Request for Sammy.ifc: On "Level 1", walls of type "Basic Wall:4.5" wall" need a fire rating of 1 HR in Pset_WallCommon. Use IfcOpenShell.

First a look at what the model holds.

```python
import ifcopenshell
import ifcopenshell.util.element

model = ifcopenshell.open("Sammy.ifc")
print(model.schema)
storey = next(s for s in model.by_type("IfcBuildingStorey") if s.Name == "Level 1")
walls = [e for e in ifcopenshell.util.element.get_decomposition(storey) if e.is_a("IfcWall")]
seen = {}
for e in walls:
    element_type = ifcopenshell.util.element.get_type(e)
    key = (element_type.Name if element_type != e and element_type else None, ifcopenshell.util.element.get_pset(e, "Pset_WallCommon", "FireRating"))
    seen[key] = seen.get(key, 0) + 1
for (name, value), count in sorted(seen.items(), key=str):
    print(count, "x", name, "|", value)
```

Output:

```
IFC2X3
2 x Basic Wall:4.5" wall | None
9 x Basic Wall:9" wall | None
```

```python
import ifcopenshell
import ifcopenshell.api.pset
import ifcopenshell.util.element

model = ifcopenshell.open("Sammy.ifc")

storey = next(s for s in model.by_type("IfcBuildingStorey") if s.Name == "Level 1")
walls = [e for e in ifcopenshell.util.element.get_decomposition(storey) if e.is_a("IfcWall")]

count = 0
for e in walls:
    element_type = ifcopenshell.util.element.get_type(e)
    if element_type in (None, e) or element_type.Name != 'Basic Wall:4.5" wall':
        continue
    # add_pset returns the element's existing set when there is one.
    pset = ifcopenshell.api.pset.add_pset(model, product=e, name="Pset_WallCommon")
    ifcopenshell.api.pset.edit_pset(model, pset=pset, properties={"FireRating": "1 HR"})
    count += 1

print(count, "walls updated")

model.write("Sammy_updated.ifc")
```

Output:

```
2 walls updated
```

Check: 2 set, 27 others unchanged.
